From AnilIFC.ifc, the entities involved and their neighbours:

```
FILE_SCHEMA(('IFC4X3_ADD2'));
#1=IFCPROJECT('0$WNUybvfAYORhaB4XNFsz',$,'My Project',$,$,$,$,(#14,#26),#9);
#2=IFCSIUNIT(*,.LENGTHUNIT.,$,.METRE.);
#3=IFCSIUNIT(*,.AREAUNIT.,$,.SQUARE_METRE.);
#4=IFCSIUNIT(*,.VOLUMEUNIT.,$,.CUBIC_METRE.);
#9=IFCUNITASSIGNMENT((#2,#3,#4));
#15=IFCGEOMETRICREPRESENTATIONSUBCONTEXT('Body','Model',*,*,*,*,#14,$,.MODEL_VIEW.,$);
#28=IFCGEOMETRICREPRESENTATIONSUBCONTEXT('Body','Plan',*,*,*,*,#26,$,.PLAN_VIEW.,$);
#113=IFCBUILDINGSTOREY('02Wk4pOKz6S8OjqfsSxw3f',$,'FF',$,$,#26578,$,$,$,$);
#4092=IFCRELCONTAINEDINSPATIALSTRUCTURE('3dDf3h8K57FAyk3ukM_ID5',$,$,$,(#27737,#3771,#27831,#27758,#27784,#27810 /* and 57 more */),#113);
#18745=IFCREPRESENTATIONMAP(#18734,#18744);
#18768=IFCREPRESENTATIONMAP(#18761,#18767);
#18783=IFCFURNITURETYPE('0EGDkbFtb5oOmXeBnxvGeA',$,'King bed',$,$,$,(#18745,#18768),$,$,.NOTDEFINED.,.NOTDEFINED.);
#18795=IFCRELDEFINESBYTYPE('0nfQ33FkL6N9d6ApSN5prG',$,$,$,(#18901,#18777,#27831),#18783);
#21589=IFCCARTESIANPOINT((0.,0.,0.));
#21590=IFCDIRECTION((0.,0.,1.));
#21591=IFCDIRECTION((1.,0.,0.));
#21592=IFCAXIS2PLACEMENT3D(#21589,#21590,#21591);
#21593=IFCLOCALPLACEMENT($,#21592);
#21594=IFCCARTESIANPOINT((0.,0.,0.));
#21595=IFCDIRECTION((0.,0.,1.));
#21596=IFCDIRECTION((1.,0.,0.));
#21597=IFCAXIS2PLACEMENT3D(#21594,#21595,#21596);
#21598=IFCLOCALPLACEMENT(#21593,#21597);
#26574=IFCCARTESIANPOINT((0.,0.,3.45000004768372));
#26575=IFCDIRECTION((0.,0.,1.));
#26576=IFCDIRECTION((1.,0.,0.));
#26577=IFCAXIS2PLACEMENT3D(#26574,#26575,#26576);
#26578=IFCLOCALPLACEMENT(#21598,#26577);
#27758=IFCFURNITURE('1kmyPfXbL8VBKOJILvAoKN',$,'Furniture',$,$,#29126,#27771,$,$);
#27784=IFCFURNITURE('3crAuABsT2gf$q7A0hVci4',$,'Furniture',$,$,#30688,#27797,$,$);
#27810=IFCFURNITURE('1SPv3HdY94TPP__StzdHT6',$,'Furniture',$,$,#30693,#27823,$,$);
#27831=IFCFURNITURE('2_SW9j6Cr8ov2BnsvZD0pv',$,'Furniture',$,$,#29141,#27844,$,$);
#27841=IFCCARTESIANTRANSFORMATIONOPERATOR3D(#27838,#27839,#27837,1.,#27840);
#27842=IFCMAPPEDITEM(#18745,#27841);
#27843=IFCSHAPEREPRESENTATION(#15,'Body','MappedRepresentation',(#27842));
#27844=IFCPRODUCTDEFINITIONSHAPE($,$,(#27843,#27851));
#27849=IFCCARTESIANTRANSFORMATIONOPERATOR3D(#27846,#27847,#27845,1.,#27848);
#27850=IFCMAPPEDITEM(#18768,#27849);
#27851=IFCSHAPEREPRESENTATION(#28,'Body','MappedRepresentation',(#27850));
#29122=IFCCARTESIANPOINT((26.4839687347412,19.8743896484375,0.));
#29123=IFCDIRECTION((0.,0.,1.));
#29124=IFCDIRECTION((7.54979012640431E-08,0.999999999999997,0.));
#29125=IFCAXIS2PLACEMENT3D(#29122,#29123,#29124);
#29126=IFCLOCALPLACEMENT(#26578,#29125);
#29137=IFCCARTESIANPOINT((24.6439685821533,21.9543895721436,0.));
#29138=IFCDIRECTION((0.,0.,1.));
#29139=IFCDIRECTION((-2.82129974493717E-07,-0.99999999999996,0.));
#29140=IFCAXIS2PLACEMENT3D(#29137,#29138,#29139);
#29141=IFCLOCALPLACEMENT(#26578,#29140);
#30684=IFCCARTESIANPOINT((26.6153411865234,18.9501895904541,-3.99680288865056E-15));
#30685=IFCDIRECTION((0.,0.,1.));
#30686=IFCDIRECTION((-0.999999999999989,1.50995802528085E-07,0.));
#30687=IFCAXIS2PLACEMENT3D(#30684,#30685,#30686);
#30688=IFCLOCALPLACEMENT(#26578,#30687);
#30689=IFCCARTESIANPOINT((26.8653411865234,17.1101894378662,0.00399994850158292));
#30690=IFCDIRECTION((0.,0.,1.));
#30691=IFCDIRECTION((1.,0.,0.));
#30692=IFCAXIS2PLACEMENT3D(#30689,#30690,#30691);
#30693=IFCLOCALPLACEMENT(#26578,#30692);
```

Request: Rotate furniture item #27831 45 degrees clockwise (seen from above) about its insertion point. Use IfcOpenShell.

```python
import ifcopenshell
import ifcopenshell.api.geometry
import ifcopenshell.util.placement

model = ifcopenshell.open("AnilIFC.ifc")

item = model.by_guid("2_SW9j6Cr8ov2BnsvZD0pv")
matrix = ifcopenshell.util.placement.get_local_placement(item.ObjectPlacement)
matrix = matrix @ ifcopenshell.util.placement.rotation(-45, "Z")
ifcopenshell.api.geometry.edit_object_placement(model, product=item, matrix=matrix, is_si=False)

print(ifcopenshell.util.placement.get_local_placement(item.ObjectPlacement).round(3) + 0.0)

model.write("AnilIFC_edited.ifc")
```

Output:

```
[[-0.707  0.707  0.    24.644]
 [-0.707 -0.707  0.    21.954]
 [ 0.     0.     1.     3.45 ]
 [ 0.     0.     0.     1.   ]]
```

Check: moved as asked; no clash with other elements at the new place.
